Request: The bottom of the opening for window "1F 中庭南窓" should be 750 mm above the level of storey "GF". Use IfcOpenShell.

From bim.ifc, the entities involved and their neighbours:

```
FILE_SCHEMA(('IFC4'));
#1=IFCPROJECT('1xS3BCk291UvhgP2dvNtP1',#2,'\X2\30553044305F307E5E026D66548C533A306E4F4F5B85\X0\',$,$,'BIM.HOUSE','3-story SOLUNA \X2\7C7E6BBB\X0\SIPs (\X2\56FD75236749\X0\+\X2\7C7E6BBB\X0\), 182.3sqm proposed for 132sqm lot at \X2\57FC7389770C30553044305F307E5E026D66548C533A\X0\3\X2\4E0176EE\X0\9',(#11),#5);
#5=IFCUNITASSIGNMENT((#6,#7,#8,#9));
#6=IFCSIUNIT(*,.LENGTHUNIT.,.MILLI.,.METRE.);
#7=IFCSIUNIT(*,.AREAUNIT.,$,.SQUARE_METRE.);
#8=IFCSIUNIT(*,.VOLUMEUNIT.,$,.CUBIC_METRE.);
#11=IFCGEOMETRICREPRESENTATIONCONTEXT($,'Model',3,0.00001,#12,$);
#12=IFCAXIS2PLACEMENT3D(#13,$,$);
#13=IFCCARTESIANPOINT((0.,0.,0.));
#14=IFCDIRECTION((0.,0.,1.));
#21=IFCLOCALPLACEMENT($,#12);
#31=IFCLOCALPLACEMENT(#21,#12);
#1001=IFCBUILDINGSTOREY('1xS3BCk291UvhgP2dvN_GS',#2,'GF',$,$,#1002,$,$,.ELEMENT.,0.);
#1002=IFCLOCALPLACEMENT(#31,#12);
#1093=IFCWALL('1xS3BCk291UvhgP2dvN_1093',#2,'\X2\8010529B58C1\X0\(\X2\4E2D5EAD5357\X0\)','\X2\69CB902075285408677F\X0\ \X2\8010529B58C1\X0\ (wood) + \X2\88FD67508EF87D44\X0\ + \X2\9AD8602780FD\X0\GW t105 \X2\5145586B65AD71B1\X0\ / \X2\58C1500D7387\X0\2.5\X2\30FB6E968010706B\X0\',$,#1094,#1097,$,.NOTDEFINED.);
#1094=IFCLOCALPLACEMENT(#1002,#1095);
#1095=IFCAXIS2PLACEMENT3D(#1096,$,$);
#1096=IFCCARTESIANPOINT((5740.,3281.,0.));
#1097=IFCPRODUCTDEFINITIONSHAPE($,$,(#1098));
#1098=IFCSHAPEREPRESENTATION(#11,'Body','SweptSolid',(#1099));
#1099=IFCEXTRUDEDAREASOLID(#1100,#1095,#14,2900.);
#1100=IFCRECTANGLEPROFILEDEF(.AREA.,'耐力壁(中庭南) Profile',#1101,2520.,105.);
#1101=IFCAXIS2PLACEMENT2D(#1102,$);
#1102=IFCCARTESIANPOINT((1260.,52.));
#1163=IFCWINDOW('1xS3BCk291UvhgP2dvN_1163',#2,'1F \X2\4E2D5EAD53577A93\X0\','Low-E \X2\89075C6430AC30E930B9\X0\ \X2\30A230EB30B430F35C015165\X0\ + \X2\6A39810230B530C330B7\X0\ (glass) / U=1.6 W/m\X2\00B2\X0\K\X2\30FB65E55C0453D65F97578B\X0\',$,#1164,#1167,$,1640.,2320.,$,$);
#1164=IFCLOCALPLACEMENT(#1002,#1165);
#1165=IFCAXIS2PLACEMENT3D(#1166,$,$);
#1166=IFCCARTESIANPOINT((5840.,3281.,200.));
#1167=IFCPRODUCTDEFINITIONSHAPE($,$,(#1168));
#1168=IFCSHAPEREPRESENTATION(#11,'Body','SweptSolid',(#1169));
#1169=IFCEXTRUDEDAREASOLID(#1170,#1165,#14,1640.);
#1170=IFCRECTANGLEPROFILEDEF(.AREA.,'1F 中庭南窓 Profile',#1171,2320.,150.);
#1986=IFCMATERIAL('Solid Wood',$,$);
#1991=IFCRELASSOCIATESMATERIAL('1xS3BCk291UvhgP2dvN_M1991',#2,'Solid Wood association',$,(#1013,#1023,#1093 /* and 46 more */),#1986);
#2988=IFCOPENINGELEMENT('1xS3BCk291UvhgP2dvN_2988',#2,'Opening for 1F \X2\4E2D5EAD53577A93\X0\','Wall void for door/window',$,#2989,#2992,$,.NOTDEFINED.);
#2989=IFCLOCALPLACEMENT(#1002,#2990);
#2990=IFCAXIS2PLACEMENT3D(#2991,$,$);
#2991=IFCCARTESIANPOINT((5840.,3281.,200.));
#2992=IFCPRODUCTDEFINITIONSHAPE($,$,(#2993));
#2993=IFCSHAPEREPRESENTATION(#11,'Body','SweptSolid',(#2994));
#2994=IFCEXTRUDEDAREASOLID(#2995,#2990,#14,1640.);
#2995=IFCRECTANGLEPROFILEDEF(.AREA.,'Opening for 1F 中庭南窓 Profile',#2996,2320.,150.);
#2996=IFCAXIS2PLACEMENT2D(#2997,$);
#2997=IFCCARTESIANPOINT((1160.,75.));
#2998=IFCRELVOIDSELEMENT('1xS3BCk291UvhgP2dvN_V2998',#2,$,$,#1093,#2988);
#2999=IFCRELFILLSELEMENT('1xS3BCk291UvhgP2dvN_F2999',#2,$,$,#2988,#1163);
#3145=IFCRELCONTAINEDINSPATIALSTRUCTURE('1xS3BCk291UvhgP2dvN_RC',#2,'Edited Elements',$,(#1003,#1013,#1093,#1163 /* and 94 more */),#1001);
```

```python
import numpy as np
import ifcopenshell
import ifcopenshell.api.geometry
import ifcopenshell.geom
import ifcopenshell.util.element
import ifcopenshell.util.placement
import ifcopenshell.util.shape
import ifcopenshell.util.unit

model = ifcopenshell.open("bim.ifc")
unit_scale = ifcopenshell.util.unit.calculate_unit_scale(model)

window = model.by_guid("1xS3BCk291UvhgP2dvN_1163")
opening = window.FillsVoids[0].RelatingOpeningElement
storey = ifcopenshell.util.element.get_container(window, ifc_class="IfcBuildingStorey")
level = ifcopenshell.util.placement.get_local_placement(storey.ObjectPlacement)[2, 3]

# The opening's origin need not be at the sill, so measure its lowest point.
shape = ifcopenshell.geom.create_shape(ifcopenshell.geom.settings(), opening)
bottom = ifcopenshell.util.shape.get_shape_bottom_elevation(shape, shape.geometry) / unit_scale
dz = level + 750.0 - bottom

shift = np.array([0.0, 0.0, dz])
# The window is not placed relative to its opening, so move both.
for product in (opening, window):
    matrix = ifcopenshell.util.placement.get_local_placement(product.ObjectPlacement)
    matrix[:3, 3] += shift
    ifcopenshell.api.geometry.edit_object_placement(model, product=product, matrix=matrix, is_si=False)

print(f"moved by {dz * unit_scale:+.3f} m")

model.write("bim_edited.ifc")
```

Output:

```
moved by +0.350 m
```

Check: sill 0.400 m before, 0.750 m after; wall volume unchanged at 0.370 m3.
